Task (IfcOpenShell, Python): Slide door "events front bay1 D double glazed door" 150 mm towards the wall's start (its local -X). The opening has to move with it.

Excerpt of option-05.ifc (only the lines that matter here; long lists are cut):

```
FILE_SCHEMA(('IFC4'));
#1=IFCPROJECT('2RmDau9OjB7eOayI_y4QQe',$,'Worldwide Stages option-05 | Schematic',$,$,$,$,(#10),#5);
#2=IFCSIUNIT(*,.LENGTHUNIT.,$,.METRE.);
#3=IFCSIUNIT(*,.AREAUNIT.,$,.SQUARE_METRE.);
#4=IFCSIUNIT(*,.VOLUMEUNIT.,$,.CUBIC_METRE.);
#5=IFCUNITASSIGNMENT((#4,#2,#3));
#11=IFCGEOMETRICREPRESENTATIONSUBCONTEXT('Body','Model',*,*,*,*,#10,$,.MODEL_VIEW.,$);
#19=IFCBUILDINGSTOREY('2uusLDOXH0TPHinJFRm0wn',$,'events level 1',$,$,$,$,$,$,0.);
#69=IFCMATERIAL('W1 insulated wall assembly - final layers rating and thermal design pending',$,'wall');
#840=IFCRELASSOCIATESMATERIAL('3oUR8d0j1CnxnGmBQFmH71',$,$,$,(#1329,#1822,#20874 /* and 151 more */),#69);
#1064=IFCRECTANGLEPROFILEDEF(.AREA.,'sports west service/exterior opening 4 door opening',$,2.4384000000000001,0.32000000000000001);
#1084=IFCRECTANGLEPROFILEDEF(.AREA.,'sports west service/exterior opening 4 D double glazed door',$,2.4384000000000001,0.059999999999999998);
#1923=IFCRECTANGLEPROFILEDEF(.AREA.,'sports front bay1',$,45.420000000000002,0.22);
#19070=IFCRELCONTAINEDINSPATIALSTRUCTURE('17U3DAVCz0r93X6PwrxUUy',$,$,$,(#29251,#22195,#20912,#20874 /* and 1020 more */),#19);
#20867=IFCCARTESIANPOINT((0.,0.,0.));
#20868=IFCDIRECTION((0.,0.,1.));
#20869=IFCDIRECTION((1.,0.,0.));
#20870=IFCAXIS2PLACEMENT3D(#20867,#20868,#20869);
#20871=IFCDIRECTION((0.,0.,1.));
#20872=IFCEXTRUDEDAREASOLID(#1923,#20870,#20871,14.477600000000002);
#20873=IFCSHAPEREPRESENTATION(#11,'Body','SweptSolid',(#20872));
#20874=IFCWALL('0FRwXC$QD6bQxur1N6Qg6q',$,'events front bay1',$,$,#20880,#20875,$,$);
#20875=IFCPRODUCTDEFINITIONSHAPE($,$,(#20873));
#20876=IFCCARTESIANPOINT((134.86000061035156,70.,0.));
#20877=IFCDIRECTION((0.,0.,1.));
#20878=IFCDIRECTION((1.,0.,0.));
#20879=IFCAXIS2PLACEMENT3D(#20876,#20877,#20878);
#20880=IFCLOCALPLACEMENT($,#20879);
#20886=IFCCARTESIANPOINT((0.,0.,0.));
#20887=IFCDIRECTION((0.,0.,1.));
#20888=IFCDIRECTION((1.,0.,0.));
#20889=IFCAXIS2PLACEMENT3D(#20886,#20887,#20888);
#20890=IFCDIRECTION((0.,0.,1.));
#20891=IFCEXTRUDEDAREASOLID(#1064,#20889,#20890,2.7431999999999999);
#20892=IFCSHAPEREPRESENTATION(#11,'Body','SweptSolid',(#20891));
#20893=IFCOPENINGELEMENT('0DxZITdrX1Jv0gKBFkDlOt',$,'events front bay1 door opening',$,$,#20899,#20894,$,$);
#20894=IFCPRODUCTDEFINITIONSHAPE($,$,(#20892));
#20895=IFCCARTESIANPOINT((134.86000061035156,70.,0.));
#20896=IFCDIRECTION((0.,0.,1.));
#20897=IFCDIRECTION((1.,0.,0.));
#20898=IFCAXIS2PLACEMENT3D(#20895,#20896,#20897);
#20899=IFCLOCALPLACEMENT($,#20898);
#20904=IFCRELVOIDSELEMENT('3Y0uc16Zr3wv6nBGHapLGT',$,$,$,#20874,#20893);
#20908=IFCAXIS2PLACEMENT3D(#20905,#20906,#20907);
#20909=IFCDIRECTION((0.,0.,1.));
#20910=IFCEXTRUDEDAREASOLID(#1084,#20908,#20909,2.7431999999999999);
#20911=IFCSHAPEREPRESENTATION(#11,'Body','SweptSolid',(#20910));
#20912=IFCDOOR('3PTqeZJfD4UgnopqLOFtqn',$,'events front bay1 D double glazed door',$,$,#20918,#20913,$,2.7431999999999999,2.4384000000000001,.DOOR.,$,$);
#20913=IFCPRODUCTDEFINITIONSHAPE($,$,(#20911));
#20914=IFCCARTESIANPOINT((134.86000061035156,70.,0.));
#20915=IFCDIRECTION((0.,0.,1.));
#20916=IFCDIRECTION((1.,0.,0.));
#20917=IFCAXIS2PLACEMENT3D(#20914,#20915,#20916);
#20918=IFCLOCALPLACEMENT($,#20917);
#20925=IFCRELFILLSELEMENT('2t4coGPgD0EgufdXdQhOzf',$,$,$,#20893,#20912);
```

```python
import ifcopenshell
import ifcopenshell.api.geometry
import ifcopenshell.util.placement
import ifcopenshell.util.unit

model = ifcopenshell.open("option-05.ifc")
unit_scale = ifcopenshell.util.unit.calculate_unit_scale(model)

door = model.by_guid("3PTqeZJfD4UgnopqLOFtqn")
opening = door.FillsVoids[0].RelatingOpeningElement
wall = opening.VoidsElements[0].RelatingBuildingElement

wall_matrix = ifcopenshell.util.placement.get_local_placement(wall.ObjectPlacement)
shift = wall_matrix[:3, 0] * -0.15 / unit_scale
before = ifcopenshell.util.placement.get_local_placement(door.ObjectPlacement)[:3, 3].copy()

# The door is not placed relative to its opening, so move both.
for product in (opening, door):
    matrix = ifcopenshell.util.placement.get_local_placement(product.ObjectPlacement)
    matrix[:3, 3] += shift
    ifcopenshell.api.geometry.edit_object_placement(model, product=product, matrix=matrix, is_si=False)

after = ifcopenshell.util.placement.get_local_placement(door.ObjectPlacement)[:3, 3]
print("door moved by", (after - before).round(3) + 0.0)

model.write("option-05_edited.ifc")
```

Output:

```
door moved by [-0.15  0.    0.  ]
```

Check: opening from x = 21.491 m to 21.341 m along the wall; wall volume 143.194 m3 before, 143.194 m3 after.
